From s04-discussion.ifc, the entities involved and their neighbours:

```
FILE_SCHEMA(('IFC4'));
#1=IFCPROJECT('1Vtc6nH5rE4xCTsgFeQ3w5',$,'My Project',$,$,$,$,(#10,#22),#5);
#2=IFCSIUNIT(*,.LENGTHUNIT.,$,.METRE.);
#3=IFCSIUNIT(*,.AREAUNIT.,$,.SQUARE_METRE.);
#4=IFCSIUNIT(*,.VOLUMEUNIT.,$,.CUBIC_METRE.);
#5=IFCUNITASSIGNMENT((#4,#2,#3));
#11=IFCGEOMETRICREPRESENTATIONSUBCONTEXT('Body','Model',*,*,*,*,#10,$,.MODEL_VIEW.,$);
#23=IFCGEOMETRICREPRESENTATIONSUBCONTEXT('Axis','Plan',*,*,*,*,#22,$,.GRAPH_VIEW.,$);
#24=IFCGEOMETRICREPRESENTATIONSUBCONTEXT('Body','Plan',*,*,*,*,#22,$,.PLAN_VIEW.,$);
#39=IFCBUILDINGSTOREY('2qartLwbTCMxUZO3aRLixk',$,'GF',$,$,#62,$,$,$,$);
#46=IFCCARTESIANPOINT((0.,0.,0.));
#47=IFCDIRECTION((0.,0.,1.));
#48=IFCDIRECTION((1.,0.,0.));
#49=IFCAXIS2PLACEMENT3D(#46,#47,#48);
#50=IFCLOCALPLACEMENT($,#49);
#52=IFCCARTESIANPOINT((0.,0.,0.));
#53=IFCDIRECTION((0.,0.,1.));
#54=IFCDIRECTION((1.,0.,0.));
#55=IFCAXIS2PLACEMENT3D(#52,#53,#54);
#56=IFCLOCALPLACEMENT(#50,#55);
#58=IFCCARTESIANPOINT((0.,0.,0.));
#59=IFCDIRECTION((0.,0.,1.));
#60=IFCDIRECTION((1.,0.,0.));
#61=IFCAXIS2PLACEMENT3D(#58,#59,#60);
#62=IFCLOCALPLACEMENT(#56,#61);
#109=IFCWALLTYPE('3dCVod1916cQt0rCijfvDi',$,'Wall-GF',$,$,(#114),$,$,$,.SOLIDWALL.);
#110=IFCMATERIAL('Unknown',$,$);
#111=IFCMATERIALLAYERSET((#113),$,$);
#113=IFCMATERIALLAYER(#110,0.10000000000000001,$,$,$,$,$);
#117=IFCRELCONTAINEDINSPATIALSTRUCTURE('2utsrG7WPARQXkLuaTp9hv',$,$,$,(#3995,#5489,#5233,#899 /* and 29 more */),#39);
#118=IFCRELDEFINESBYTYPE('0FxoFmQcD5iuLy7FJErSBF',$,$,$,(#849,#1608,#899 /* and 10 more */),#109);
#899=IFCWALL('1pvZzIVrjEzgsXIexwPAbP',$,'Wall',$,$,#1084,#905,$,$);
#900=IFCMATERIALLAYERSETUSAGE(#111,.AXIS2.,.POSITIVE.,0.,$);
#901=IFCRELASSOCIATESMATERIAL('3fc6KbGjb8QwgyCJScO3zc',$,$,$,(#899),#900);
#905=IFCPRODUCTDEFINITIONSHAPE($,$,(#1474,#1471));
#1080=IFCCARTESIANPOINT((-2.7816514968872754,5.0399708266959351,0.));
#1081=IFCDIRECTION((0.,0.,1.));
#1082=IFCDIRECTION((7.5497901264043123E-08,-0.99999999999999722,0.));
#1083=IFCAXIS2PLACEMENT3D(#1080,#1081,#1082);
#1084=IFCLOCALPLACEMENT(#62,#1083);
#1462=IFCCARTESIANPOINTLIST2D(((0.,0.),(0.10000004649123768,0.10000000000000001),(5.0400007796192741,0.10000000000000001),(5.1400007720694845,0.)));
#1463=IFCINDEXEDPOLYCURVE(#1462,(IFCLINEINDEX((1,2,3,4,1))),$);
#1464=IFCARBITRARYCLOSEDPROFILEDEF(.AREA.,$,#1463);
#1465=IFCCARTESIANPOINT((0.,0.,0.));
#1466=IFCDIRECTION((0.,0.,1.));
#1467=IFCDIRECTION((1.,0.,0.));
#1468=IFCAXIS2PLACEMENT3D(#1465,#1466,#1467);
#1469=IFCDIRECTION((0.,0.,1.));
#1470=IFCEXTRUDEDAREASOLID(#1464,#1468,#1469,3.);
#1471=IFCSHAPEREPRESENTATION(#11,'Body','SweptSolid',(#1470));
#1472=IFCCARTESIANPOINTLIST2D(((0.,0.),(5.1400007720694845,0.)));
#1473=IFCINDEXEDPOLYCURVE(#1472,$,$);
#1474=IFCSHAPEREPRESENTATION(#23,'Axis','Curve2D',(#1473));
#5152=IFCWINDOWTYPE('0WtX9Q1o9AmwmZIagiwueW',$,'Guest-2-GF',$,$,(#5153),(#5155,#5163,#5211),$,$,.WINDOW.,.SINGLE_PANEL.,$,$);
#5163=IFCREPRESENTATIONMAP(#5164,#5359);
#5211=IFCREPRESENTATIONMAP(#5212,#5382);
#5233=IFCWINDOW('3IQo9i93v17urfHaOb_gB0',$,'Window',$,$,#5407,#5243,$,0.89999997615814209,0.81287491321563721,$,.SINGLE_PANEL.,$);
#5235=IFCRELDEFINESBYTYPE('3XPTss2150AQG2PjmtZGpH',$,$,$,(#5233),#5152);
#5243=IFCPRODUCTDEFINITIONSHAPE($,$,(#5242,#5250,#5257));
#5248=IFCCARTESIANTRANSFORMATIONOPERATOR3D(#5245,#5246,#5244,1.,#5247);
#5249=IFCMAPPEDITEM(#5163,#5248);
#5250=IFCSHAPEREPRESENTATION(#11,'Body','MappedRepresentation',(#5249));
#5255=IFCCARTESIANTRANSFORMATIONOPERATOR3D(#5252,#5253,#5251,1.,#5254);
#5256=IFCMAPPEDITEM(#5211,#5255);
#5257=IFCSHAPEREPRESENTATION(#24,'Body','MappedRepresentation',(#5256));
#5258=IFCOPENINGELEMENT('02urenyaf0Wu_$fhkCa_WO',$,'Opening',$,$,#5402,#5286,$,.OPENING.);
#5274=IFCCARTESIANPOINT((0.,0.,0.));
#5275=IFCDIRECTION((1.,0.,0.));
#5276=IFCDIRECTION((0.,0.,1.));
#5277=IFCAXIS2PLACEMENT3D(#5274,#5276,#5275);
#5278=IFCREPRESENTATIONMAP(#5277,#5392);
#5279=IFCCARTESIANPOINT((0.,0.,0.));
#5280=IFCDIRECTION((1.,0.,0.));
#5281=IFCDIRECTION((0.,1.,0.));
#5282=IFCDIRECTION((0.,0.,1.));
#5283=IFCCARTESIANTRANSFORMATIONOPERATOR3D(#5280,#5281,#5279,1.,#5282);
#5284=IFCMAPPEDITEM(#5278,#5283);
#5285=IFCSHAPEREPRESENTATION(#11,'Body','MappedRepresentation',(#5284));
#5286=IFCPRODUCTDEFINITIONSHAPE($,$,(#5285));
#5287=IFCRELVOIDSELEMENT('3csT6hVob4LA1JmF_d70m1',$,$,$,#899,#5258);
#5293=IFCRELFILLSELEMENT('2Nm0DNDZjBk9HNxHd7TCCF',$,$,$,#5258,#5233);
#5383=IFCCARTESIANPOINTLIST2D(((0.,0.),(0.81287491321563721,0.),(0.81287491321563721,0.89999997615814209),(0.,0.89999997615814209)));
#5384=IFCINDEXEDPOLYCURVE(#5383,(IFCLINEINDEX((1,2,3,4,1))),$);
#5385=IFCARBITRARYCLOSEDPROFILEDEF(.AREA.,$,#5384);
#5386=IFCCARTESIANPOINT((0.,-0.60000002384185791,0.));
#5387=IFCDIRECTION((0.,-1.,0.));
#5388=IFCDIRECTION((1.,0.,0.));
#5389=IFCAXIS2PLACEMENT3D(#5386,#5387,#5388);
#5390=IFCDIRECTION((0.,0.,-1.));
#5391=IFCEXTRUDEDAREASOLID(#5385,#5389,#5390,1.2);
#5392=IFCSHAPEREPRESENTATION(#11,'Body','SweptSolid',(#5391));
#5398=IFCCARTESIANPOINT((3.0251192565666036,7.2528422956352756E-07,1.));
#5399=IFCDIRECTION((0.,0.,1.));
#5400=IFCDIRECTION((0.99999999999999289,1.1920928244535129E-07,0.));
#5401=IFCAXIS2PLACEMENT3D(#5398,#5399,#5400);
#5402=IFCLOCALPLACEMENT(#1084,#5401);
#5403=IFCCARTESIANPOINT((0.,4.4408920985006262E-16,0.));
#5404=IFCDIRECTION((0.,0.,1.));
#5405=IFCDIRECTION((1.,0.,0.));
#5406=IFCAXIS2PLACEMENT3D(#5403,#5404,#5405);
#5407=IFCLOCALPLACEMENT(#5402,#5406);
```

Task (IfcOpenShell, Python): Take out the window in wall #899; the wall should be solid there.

```python
import ifcopenshell
import ifcopenshell.api.feature
import ifcopenshell.api.root
import ifcopenshell.geom
import ifcopenshell.util.shape

model = ifcopenshell.open("s04-discussion.ifc")
settings = ifcopenshell.geom.settings()


def volume(element):
    """Net volume in cubic metres, openings subtracted."""
    shape = ifcopenshell.geom.create_shape(settings, element)
    return ifcopenshell.util.shape.get_volume(shape.geometry)


window = model.by_guid("3IQo9i93v17urfHaOb_gB0")
opening = window.FillsVoids[0].RelatingOpeningElement
wall = opening.VoidsElements[0].RelatingBuildingElement
before = volume(wall)

ifcopenshell.api.root.remove_product(model, product=window)
ifcopenshell.api.feature.remove_feature(model, feature=opening)

after = volume(wall)

print(f"wall volume {before:.3f} -> {after:.3f} m3")

model.write("s04-discussion_v2.ifc")
```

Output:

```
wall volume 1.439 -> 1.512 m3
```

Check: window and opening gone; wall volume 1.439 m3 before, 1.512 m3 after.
